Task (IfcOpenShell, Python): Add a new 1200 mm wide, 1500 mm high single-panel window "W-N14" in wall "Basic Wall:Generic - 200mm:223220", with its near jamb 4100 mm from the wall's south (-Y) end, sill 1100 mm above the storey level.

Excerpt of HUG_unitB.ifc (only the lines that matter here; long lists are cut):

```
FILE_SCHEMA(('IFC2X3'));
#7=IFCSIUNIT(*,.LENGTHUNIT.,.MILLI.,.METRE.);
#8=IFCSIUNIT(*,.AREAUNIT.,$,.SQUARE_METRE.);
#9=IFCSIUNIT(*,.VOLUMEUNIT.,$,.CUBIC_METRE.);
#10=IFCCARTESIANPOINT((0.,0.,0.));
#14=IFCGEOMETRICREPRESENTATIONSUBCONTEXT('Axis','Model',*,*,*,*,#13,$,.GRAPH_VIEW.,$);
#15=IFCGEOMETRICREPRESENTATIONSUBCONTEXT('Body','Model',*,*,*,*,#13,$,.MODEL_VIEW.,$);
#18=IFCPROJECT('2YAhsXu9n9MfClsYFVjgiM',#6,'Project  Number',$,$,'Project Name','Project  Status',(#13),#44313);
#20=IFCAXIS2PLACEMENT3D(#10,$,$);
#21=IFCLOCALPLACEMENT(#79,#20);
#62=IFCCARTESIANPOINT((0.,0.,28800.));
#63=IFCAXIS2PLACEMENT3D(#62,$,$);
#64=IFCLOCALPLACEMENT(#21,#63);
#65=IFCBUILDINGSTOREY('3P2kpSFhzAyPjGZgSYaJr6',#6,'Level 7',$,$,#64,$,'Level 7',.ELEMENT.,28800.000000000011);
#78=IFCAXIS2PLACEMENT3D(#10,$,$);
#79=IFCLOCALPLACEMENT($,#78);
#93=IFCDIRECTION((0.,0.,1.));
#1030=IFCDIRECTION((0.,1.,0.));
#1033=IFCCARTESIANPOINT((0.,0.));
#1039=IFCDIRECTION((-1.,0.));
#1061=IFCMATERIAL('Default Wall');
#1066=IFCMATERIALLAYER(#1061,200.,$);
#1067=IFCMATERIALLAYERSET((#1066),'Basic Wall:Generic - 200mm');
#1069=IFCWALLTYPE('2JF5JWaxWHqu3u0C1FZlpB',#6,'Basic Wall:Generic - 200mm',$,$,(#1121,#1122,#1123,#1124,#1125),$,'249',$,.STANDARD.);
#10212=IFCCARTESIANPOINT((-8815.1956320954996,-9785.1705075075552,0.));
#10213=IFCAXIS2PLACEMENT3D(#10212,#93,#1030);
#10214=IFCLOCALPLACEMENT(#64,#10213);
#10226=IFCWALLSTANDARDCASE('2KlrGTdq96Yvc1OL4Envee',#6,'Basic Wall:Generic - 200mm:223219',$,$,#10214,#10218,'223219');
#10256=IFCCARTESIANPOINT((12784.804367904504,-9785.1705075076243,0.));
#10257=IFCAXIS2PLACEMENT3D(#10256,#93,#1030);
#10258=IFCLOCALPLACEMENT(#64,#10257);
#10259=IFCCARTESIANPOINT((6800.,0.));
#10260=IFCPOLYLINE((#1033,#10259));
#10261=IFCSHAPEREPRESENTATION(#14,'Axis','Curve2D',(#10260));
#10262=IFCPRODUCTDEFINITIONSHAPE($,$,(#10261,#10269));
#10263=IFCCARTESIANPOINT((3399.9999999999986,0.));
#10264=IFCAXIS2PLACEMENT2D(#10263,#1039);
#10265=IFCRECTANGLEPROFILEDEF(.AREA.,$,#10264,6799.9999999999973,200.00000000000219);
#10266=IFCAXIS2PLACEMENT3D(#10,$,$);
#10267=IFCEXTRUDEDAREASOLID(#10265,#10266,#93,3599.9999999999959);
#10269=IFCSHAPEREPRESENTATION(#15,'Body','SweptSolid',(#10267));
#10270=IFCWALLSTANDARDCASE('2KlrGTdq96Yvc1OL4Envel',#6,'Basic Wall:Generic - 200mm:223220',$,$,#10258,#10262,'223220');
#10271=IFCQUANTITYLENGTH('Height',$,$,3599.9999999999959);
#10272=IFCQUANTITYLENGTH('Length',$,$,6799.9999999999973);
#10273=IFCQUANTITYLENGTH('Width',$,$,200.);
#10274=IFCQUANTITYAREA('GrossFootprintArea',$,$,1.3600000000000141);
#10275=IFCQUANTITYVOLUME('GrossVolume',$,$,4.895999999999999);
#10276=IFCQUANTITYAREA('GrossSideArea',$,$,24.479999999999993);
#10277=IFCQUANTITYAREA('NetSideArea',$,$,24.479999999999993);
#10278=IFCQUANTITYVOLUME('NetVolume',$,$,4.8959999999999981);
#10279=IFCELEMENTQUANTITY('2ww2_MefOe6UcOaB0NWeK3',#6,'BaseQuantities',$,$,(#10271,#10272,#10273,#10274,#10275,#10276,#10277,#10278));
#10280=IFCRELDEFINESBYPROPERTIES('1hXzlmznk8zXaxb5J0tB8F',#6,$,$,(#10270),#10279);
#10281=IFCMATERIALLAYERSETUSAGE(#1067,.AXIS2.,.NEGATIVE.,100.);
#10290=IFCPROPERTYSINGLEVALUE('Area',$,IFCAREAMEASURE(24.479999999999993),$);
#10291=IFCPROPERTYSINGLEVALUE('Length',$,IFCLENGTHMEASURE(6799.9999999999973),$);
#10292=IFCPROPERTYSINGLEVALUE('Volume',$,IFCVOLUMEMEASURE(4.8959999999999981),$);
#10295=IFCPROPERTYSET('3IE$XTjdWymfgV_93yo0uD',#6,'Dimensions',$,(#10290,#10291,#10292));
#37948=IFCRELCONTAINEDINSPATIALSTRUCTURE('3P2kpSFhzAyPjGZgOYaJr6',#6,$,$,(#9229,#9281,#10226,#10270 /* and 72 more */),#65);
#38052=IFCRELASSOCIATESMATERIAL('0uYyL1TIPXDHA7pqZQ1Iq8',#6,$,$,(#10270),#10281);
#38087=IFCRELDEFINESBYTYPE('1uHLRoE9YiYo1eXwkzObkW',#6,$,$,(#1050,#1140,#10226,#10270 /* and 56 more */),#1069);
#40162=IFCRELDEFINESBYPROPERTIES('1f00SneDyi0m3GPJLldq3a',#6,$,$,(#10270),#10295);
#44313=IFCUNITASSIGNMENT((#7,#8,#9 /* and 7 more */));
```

```python
import numpy as np
import ifcopenshell
import ifcopenshell.api.feature
import ifcopenshell.api.geometry
import ifcopenshell.api.pset
import ifcopenshell.api.root
import ifcopenshell.api.spatial
import ifcopenshell.api.type
import ifcopenshell.geom
import ifcopenshell.util.element
import ifcopenshell.util.placement
import ifcopenshell.util.representation
import ifcopenshell.util.shape
import ifcopenshell.util.unit

model = ifcopenshell.open("HUG_unitB.ifc")
unit_scale = ifcopenshell.util.unit.calculate_unit_scale(model)
area_scale = ifcopenshell.util.unit.calculate_unit_scale(model, "AREAUNIT")
volume_scale = ifcopenshell.util.unit.calculate_unit_scale(model, "VOLUMEUNIT")
settings = ifcopenshell.geom.settings()


def volume(element):
    """Net volume in cubic metres, openings subtracted."""
    shape = ifcopenshell.geom.create_shape(settings, element)
    return ifcopenshell.util.shape.get_volume(shape.geometry)


wall = model.by_guid("2KlrGTdq96Yvc1OL4Envel")
storey = ifcopenshell.util.element.get_container(wall, ifc_class="IfcBuildingStorey")
context = ifcopenshell.util.representation.get_context(model, "Model", "Body", "MODEL_VIEW")
before = volume(wall)

width, height, from_end, sill = 1.2, 1.5, 4.1, 1.1  # metres

# The wall runs along its own X axis, and the end named is its -X end.
wall_shape = ifcopenshell.geom.create_shape(settings, wall)
x, y, z = ifcopenshell.util.shape.get_vertices(wall_shape.geometry).T
start = x.min() + from_end
face, thickness = float(y.min()), float(y.max() - y.min())
wall_matrix = ifcopenshell.util.placement.get_local_placement(wall.ObjectPlacement)
level = ifcopenshell.util.placement.get_local_placement(storey.ObjectPlacement)[2, 3]


def in_wall(x, y):
    """Placement at x, y metres in the wall's axes, at sill height."""
    matrix = wall_matrix.copy()
    matrix[:, 3] = wall_matrix @ np.array([x / unit_scale, y / unit_scale, 0.0, 1.0])
    matrix[2, 3] = level + sill / unit_scale
    return matrix


# Opening: a box that overshoots both wall faces by 50 mm.
opening = ifcopenshell.api.root.create_entity(model, ifc_class="IfcOpeningElement")
box = ifcopenshell.api.geometry.add_wall_representation(
    model, context=context, length=width, height=height, thickness=thickness + 0.1
)
ifcopenshell.api.geometry.assign_representation(model, product=opening, representation=box)
ifcopenshell.api.geometry.edit_object_placement(model, product=opening, matrix=in_wall(start, face - 0.05), is_si=False)
ifcopenshell.api.feature.add_feature(model, feature=opening, element=wall)

window = ifcopenshell.api.root.create_entity(model, ifc_class="IfcWindow", name="W-N14")
window.OverallWidth, window.OverallHeight = width / unit_scale, height / unit_scale
body = ifcopenshell.api.geometry.add_window_representation(
    model,
    context=context,
    overall_width=window.OverallWidth,
    overall_height=window.OverallHeight,
    partition_type="SINGLE_PANEL",
)
ifcopenshell.api.geometry.assign_representation(model, product=window, representation=body)
ifcopenshell.api.spatial.assign_container(model, products=[window], relating_structure=storey)
fills = ifcopenshell.api.feature.add_filling(model, opening=opening, element=window)
fills.OwnerHistory = window.OwnerHistory  # required in IFC2X3

# IFC2X3 keeps the operation on the window style.
style = ifcopenshell.api.root.create_entity(model, ifc_class="IfcWindowStyle", name="W-N14")
style.OperationType, style.ConstructionType = "SINGLE_PANEL", "NOTDEFINED"
style.ParameterTakesPrecedence = style.Sizeable = False
ifcopenshell.api.type.assign_type(model, related_objects=[window], relating_type=style)

# Centre the window in the wall's thickness.
ifcopenshell.api.geometry.edit_object_placement(model, product=window, matrix=in_wall(start, face), is_si=False)
window_shape = ifcopenshell.geom.create_shape(settings, window)
depth = ifcopenshell.util.shape.get_vertices(window_shape.geometry)[:, 1]
offset = face + thickness / 2 - (depth.min() + depth.max()) / 2
ifcopenshell.api.geometry.edit_object_placement(model, product=window, matrix=in_wall(start, offset), is_si=False)

after = volume(wall)

# Update the wall's stored quantities.
qto = model.by_id(ifcopenshell.util.element.get_pset(wall, "BaseQuantities", should_inherit=False)["id"])
ifcopenshell.api.pset.edit_qto(model, qto=qto, properties={
    "NetSideArea": after / thickness / area_scale,
    "NetVolume": after / volume_scale,
})
pset = model.by_id(ifcopenshell.util.element.get_pset(wall, "Dimensions", should_inherit=False)["id"])
ifcopenshell.api.pset.edit_pset(model, pset=pset, properties={
    "Area": model.create_entity("IfcAreaMeasure", after / thickness / area_scale),
    "Volume": model.create_entity("IfcVolumeMeasure", after / volume_scale),
})

print(f"wall volume {before:.3f} -> {after:.3f} m3")

model.write("HUG_unitB-out.ifc")
```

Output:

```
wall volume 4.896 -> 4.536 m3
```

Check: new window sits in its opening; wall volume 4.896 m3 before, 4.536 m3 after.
